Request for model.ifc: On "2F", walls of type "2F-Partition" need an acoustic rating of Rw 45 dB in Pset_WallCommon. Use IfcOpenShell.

First a look at what the model holds.

```python
import ifcopenshell
import ifcopenshell.util.element

model = ifcopenshell.open("model.ifc")
print(model.schema)
storey = next(s for s in model.by_type("IfcBuildingStorey") if s.Name == "2F")
walls = [e for e in ifcopenshell.util.element.get_decomposition(storey) if e.is_a("IfcWall")]
seen = {}
for e in walls:
    element_type = ifcopenshell.util.element.get_type(e)
    key = (element_type.Name if element_type != e and element_type else None, ifcopenshell.util.element.get_pset(e, "Pset_WallCommon", "AcousticRating"))
    seen[key] = seen.get(key, 0) + 1
for (name, value), count in sorted(seen.items(), key=str):
    print(count, "x", name, "|", value)
```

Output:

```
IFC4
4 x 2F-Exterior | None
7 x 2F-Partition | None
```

```python
import ifcopenshell
import ifcopenshell.api.pset
import ifcopenshell.util.element

model = ifcopenshell.open("model.ifc")

storey = next(s for s in model.by_type("IfcBuildingStorey") if s.Name == "2F")
walls = [e for e in ifcopenshell.util.element.get_decomposition(storey) if e.is_a("IfcWall")]

count = 0
for e in walls:
    element_type = ifcopenshell.util.element.get_type(e)
    if element_type in (None, e) or element_type.Name != "2F-Partition":
        continue
    # add_pset returns the element's existing set when there is one.
    pset = ifcopenshell.api.pset.add_pset(model, product=e, name="Pset_WallCommon")
    ifcopenshell.api.pset.edit_pset(model, pset=pset, properties={"AcousticRating": "Rw 45 dB"})
    count += 1

print(count, "walls updated")

model.write("model_rev.ifc")
```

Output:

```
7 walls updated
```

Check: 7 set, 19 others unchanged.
